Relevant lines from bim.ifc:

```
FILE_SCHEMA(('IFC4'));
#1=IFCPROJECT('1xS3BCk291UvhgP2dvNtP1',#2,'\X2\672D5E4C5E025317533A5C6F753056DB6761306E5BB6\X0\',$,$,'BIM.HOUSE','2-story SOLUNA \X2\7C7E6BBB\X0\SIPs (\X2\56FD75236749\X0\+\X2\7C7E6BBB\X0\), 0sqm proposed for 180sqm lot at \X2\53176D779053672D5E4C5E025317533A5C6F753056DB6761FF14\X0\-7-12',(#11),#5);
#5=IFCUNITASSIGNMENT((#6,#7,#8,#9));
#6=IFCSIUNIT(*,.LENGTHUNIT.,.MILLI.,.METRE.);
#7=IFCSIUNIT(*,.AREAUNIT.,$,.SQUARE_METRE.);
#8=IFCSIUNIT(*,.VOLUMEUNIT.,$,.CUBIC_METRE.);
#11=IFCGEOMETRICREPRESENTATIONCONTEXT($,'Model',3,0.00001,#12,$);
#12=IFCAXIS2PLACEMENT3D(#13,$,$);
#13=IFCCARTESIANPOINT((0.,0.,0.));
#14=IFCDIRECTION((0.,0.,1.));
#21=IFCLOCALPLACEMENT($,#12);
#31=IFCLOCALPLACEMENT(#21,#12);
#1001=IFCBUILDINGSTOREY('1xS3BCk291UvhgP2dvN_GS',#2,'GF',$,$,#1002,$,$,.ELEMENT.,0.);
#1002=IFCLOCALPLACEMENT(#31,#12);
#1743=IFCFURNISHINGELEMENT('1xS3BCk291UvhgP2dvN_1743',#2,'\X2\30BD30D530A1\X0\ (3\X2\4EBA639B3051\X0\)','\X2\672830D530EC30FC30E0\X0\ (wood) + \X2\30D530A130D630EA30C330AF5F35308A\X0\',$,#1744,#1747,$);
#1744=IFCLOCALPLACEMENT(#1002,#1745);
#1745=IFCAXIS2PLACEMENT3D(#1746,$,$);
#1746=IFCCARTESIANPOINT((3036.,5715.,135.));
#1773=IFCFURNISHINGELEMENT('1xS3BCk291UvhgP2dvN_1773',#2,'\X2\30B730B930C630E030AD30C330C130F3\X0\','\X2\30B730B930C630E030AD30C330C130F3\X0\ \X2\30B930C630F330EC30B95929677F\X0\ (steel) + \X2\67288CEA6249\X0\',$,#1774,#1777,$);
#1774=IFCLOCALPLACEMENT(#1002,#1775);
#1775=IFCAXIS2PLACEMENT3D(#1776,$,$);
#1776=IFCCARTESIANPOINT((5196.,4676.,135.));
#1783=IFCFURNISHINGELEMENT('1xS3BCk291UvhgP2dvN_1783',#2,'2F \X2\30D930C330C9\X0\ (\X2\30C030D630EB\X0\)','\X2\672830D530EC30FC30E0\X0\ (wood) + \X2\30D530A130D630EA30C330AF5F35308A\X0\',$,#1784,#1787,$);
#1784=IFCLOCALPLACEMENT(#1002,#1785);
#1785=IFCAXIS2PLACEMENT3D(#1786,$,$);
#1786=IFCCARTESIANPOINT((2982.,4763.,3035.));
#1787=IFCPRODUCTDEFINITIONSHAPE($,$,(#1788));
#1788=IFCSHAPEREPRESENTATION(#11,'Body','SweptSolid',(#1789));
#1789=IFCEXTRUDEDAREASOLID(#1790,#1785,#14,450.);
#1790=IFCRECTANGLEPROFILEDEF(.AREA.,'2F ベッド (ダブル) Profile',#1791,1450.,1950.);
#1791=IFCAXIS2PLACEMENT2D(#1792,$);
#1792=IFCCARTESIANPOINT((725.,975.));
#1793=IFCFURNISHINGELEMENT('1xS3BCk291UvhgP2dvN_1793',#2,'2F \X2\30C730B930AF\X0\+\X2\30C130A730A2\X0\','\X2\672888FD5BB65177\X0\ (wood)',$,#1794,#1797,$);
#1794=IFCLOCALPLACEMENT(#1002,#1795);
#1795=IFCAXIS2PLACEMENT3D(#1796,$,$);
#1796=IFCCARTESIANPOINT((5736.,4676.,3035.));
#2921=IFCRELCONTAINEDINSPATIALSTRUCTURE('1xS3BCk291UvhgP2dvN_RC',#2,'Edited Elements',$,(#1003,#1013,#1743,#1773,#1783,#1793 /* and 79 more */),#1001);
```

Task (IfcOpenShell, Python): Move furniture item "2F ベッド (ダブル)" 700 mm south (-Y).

```python
import ifcopenshell
import ifcopenshell.api.geometry
import ifcopenshell.util.placement

model = ifcopenshell.open("bim.ifc")

item = model.by_guid("1xS3BCk291UvhgP2dvN_1783")
matrix = ifcopenshell.util.placement.get_local_placement(item.ObjectPlacement)
matrix[1, 3] -= 700.0
ifcopenshell.api.geometry.edit_object_placement(model, product=item, matrix=matrix, is_si=False)

print(ifcopenshell.util.placement.get_local_placement(item.ObjectPlacement).round(3) + 0.0)

model.write("bim_rev.ifc")
```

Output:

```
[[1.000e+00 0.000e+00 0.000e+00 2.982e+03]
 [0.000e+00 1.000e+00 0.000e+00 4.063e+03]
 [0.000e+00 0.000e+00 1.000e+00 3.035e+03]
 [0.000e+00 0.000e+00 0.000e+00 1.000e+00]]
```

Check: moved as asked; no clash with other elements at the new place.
